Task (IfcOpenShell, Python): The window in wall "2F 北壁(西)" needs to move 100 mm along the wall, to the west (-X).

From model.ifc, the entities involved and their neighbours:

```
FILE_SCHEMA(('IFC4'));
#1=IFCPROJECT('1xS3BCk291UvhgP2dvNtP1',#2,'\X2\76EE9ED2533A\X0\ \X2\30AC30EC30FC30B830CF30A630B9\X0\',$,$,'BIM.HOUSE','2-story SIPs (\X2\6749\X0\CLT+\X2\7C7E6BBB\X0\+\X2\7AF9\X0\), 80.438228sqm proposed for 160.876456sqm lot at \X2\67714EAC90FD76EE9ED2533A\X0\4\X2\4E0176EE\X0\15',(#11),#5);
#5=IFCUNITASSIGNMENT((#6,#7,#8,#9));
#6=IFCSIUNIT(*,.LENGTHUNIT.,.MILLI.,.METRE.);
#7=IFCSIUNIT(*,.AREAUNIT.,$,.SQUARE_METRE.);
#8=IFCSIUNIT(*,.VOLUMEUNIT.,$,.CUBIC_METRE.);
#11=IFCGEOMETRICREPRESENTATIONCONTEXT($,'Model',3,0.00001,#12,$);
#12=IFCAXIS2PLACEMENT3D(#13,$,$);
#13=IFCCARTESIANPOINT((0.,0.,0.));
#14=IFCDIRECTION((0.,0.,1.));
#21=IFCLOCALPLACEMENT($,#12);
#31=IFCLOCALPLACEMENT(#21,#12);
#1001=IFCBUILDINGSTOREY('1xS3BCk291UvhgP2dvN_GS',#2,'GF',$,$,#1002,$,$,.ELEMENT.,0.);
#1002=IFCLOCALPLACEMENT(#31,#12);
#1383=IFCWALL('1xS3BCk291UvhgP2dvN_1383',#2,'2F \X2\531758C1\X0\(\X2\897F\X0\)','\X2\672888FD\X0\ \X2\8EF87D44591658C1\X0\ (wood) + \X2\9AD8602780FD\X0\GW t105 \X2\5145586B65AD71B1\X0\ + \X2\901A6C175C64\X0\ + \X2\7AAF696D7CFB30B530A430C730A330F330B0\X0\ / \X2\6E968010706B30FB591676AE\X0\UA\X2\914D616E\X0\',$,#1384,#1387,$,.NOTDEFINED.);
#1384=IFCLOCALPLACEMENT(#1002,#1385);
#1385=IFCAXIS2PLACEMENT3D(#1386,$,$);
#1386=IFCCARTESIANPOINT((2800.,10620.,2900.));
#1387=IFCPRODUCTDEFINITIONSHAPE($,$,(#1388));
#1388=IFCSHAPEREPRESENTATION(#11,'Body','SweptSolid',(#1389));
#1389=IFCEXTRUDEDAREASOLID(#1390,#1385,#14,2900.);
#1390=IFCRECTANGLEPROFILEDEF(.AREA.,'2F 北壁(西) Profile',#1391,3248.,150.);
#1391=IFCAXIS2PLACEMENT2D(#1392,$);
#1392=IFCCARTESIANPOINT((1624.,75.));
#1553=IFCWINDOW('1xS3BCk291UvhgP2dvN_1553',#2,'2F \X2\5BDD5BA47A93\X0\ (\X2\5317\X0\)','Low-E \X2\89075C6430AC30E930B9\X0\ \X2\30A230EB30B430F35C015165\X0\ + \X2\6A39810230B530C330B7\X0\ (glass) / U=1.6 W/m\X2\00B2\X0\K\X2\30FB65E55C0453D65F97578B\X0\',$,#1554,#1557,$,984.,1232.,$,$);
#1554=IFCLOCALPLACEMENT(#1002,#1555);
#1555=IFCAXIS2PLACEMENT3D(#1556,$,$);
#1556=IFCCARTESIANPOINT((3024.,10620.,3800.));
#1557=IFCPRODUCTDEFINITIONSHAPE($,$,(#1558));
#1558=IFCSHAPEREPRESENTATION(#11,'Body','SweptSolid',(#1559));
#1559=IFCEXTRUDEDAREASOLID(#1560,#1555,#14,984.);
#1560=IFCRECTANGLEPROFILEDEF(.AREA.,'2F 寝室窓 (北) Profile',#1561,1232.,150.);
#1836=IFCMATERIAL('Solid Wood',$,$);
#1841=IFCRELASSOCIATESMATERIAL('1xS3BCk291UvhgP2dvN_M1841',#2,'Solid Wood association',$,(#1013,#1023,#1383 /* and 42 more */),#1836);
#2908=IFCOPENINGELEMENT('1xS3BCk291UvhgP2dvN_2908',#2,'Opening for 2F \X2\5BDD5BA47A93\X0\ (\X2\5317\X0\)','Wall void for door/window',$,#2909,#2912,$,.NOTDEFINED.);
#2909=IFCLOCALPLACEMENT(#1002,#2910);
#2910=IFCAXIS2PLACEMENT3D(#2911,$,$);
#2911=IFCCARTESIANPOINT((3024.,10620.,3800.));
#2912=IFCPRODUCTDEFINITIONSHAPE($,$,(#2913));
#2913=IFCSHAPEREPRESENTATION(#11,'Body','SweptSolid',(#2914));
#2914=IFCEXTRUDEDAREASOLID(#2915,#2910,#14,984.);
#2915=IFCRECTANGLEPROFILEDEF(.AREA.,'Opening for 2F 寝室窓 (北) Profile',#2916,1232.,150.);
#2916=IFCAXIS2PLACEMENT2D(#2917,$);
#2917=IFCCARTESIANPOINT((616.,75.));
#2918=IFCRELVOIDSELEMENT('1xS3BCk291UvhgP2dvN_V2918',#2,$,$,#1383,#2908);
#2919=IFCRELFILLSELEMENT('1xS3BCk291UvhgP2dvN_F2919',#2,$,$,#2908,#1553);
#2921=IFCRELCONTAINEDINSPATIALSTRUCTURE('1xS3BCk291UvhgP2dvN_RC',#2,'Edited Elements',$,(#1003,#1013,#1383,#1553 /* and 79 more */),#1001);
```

```python
import ifcopenshell
import ifcopenshell.api.geometry
import ifcopenshell.util.placement

model = ifcopenshell.open("model.ifc")

window = model.by_guid("1xS3BCk291UvhgP2dvN_1553")
opening = window.FillsVoids[0].RelatingOpeningElement
wall = opening.VoidsElements[0].RelatingBuildingElement

wall_matrix = ifcopenshell.util.placement.get_local_placement(wall.ObjectPlacement)
shift = wall_matrix[:3, 0] * -100.0
before = ifcopenshell.util.placement.get_local_placement(window.ObjectPlacement)[:3, 3].copy()

# The window is not placed relative to its opening, so move both.
for product in (opening, window):
    matrix = ifcopenshell.util.placement.get_local_placement(product.ObjectPlacement)
    matrix[:3, 3] += shift
    ifcopenshell.api.geometry.edit_object_placement(model, product=product, matrix=matrix, is_si=False)

after = ifcopenshell.util.placement.get_local_placement(window.ObjectPlacement)[:3, 3]
print("window moved by", (after - before).round(3) + 0.0)

model.write("model_v2.ifc")
```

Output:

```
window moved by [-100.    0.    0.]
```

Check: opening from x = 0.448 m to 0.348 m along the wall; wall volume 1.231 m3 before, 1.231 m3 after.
